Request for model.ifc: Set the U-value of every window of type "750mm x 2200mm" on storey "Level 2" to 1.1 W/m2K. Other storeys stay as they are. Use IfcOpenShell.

First a look at what the model holds.

```python
import ifcopenshell
import ifcopenshell.util.element

model = ifcopenshell.open("model.ifc")
print(model.schema)
storey = next(s for s in model.by_type("IfcBuildingStorey") if s.Name == "Level 2")
windows = [e for e in ifcopenshell.util.element.get_decomposition(storey) if e.is_a("IfcWindow")]
seen = {}
for e in windows:
    element_type = ifcopenshell.util.element.get_type(e)
    key = (element_type.Name if element_type != e and element_type else None, ifcopenshell.util.element.get_pset(e, "Pset_WindowCommon", "ThermalTransmittance"))
    seen[key] = seen.get(key, 0) + 1
for (name, value), count in sorted(seen.items(), key=str):
    print(count, "x", name, "|", value)
```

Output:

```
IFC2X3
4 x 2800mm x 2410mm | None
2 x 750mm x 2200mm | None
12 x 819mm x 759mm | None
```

```python
import ifcopenshell
import ifcopenshell.api.pset
import ifcopenshell.util.element

model = ifcopenshell.open("model.ifc")

storey = next(s for s in model.by_type("IfcBuildingStorey") if s.Name == "Level 2")
windows = [e for e in ifcopenshell.util.element.get_decomposition(storey) if e.is_a("IfcWindow")]

count = 0
for e in windows:
    element_type = ifcopenshell.util.element.get_type(e)
    if element_type in (None, e) or element_type.Name != "750mm x 2200mm":
        continue
    # add_pset returns the element's existing set when there is one.
    pset = ifcopenshell.api.pset.add_pset(model, product=e, name="Pset_WindowCommon")
    ifcopenshell.api.pset.edit_pset(model, pset=pset, properties={"ThermalTransmittance": 1.1})
    count += 1

print(count, "windows updated")

model.write("model_edited.ifc")
```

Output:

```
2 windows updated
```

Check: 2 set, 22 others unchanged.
